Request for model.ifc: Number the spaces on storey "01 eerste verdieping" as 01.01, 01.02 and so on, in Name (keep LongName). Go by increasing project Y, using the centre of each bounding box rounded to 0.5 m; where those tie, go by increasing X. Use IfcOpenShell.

First a look at what the model holds.

```python
import ifcopenshell
import ifcopenshell.util.element
import ifcopenshell.util.placement

model = ifcopenshell.open("model.ifc")
print(model.schema)
storey = next(s for s in model.by_type("IfcBuildingStorey") if s.Name == "01 eerste verdieping")
spaces = [e for e in ifcopenshell.util.element.get_decomposition(storey) if e.is_a("IfcSpace")]
for e in sorted(spaces, key=lambda e: e.id()):
    origin = ifcopenshell.util.placement.get_local_placement(e.ObjectPlacement)[:3, 3]
    print(e.id(), e.Name, e.LongName, origin.round(2) + 0.0, sep=" | ")
```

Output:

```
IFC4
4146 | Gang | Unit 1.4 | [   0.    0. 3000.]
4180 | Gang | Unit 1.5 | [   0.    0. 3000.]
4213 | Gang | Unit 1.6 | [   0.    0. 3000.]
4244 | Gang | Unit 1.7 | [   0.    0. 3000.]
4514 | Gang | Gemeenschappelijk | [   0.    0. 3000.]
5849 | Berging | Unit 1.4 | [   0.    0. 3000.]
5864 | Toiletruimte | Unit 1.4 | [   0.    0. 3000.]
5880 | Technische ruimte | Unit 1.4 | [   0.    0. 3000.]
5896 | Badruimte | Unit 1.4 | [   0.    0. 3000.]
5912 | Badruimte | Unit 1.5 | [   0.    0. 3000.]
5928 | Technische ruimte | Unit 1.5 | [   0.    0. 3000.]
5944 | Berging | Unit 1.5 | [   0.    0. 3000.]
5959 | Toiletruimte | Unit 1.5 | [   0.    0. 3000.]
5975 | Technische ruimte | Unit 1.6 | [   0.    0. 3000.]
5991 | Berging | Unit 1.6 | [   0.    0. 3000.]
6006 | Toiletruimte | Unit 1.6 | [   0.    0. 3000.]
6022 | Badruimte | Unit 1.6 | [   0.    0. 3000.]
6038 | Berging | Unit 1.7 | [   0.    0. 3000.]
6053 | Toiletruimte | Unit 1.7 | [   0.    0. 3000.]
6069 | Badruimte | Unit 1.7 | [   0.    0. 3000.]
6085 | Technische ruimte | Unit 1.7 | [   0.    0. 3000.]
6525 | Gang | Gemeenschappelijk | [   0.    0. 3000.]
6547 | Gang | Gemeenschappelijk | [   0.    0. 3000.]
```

```python
import ifcopenshell
import ifcopenshell.geom
import ifcopenshell.util.element
import ifcopenshell.util.shape

model = ifcopenshell.open("model.ifc")
settings = ifcopenshell.geom.settings()
settings.set("use-world-coords", True)


def centre(element):
    shape = ifcopenshell.geom.create_shape(settings, element)
    return ifcopenshell.util.shape.get_bbox_centroid(shape.geometry)


storey = next(s for s in model.by_type("IfcBuildingStorey") if s.Name == "01 eerste verdieping")
spaces = [e for e in ifcopenshell.util.element.get_decomposition(storey) if e.is_a("IfcSpace")]

# Insertion points can sit at a corner or the storey origin, so sort by the geometry (in metres).
centres = {e: centre(e) for e in spaces}
spaces.sort(key=lambda e: (round(centres[e][1] / 0.5), centres[e][0]))

for i, e in enumerate(spaces, start=1):
    number = f"01.{i:02d}"
    e.Name = number
    print(e.id(), number)

model.write("model_updated.ifc")
```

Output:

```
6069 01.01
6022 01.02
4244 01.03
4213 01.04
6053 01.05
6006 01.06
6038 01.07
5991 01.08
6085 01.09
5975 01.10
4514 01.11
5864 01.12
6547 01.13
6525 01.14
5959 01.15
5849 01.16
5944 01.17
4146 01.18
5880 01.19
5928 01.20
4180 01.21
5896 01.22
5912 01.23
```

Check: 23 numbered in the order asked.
